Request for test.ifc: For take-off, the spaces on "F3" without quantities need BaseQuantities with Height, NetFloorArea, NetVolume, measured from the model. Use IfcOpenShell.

First a look at what the model holds.

```python
import ifcopenshell
import ifcopenshell.util.element
import ifcopenshell.util.unit

model = ifcopenshell.open("test.ifc")
print(model.schema)
for unit_type in ("LENGTHUNIT", "AREAUNIT", "VOLUMEUNIT"):
    print(unit_type, ifcopenshell.util.unit.calculate_unit_scale(model, unit_type))
storey = next(s for s in model.by_type("IfcBuildingStorey") if s.Name == "F3")
spaces = [e for e in ifcopenshell.util.element.get_decomposition(storey) if e.is_a("IfcSpace")]
for e in sorted(spaces, key=lambda e: e.id()):
    print(e.id(), e.is_a(), e.Name, list(ifcopenshell.util.element.get_psets(e, qtos_only=True)), sep=" | ")
```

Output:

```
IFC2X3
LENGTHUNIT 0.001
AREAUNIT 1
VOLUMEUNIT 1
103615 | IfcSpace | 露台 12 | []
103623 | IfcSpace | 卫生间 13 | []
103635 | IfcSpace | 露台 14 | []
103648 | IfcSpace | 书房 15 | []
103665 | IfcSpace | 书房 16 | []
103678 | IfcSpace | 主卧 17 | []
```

```python
import ifcopenshell
import ifcopenshell.api.pset
import ifcopenshell.geom
import ifcopenshell.util.element
import ifcopenshell.util.shape
import ifcopenshell.util.unit

model = ifcopenshell.open("test.ifc")
unit_scale = ifcopenshell.util.unit.calculate_unit_scale(model)
area_scale = ifcopenshell.util.unit.calculate_unit_scale(model, "AREAUNIT")
volume_scale = ifcopenshell.util.unit.calculate_unit_scale(model, "VOLUMEUNIT")
settings = ifcopenshell.geom.settings()

storey = next(s for s in model.by_type("IfcBuildingStorey") if s.Name == "F3")
spaces = [e for e in ifcopenshell.util.element.get_decomposition(storey) if e.is_a("IfcSpace")]

for e in sorted(spaces, key=lambda e: e.id()):
    if ifcopenshell.util.element.get_psets(e, qtos_only=True, should_inherit=False):
        continue
    # Geometry comes back in metres, in the element's own axes.
    shape = ifcopenshell.geom.create_shape(settings, e)
    values = {
        "Height": ifcopenshell.util.shape.get_z(shape.geometry) / unit_scale,
        "NetFloorArea": ifcopenshell.util.shape.get_footprint_area(shape.geometry) / area_scale,
        "NetVolume": ifcopenshell.util.shape.get_volume(shape.geometry) / volume_scale,
    }
    qto = ifcopenshell.api.pset.add_qto(model, product=e, name="BaseQuantities")
    ifcopenshell.api.pset.edit_qto(model, qto=qto, properties=values)
    print(e.id(), {k: round(v, 3) for k, v in values.items()})

model.write("test_updated.ifc")
```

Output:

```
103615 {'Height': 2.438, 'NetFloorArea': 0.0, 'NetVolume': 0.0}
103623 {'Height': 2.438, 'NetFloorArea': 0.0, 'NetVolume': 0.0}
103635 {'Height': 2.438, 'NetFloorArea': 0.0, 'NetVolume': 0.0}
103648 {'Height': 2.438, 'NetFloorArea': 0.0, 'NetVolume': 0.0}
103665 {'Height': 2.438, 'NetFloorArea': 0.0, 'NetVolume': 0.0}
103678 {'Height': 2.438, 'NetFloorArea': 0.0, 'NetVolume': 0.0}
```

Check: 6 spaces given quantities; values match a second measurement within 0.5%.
